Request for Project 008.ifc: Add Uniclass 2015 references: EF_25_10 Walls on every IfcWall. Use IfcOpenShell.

First a look at what the model holds.

```python
import ifcopenshell

model = ifcopenshell.open("Project 008.ifc")
print(model.schema)
print("classifications:", [c.Name for c in model.by_type("IfcClassification")])
for ifc_class in ("IfcDoor", "IfcRoof", "IfcStair", "IfcWall", "IfcWindow"):
    print(ifc_class, len(model.by_type(ifc_class)))
```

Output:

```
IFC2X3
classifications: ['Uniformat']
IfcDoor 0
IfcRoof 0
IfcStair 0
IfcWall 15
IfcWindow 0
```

```python
import ifcopenshell
import ifcopenshell.api.classification

model = ifcopenshell.open("Project 008.ifc")

# IFC2X3 requires Source and Edition and has no link from the project to the system.
system = model.create_entity("IfcClassification", Source="NBS", Edition="2015", Name="Uniclass 2015")

codes = {
    "IfcWall": ("EF_25_10", "Walls"),
}
for ifc_class, (code, name) in codes.items():
    products = model.by_type(ifc_class)
    ifcopenshell.api.classification.add_reference(
        model, products=products, classification=system, identification=code, name=name
    )
    print(code, len(products))

model.write("Project 008_v2.ifc")
```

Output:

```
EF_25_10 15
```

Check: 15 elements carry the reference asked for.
